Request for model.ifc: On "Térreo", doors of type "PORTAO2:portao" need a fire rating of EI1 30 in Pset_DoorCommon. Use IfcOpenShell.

First a look at what the model holds.

```python
import ifcopenshell
import ifcopenshell.util.element

model = ifcopenshell.open("model.ifc")
print(model.schema)
storey = next(s for s in model.by_type("IfcBuildingStorey") if s.Name == "Térreo")
doors = [e for e in ifcopenshell.util.element.get_decomposition(storey) if e.is_a("IfcDoor")]
seen = {}
for e in doors:
    element_type = ifcopenshell.util.element.get_type(e)
    key = (element_type.Name if element_type != e and element_type else None, ifcopenshell.util.element.get_pset(e, "Pset_DoorCommon", "FireRating"))
    seen[key] = seen.get(key, 0) + 1
for (name, value), count in sorted(seen.items(), key=str):
    print(count, "x", name, "|", value)
```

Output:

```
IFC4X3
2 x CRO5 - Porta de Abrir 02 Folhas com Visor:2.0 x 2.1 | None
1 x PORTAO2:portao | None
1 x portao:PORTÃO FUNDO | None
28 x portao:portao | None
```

```python
import ifcopenshell
import ifcopenshell.api.pset
import ifcopenshell.util.element

model = ifcopenshell.open("model.ifc")

storey = next(s for s in model.by_type("IfcBuildingStorey") if s.Name == "Térreo")
doors = [e for e in ifcopenshell.util.element.get_decomposition(storey) if e.is_a("IfcDoor")]

count = 0
for e in doors:
    element_type = ifcopenshell.util.element.get_type(e)
    if element_type in (None, e) or element_type.Name != "PORTAO2:portao":
        continue
    # add_pset returns the element's existing set when there is one.
    pset = ifcopenshell.api.pset.add_pset(model, product=e, name="Pset_DoorCommon")
    ifcopenshell.api.pset.edit_pset(model, pset=pset, properties={"FireRating": "EI1 30"})
    count += 1

print(count, "doors updated")

model.write("model_v2.ifc")
```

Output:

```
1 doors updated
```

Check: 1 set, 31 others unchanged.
